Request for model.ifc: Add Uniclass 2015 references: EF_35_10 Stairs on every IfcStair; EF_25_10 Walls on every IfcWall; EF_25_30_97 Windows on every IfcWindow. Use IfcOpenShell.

First a look at what the model holds.

```python
import ifcopenshell

model = ifcopenshell.open("model.ifc")
print(model.schema)
print("classifications:", [c.Name for c in model.by_type("IfcClassification")])
for ifc_class in ("IfcDoor", "IfcRoof", "IfcStair", "IfcWall", "IfcWindow"):
    print(ifc_class, len(model.by_type(ifc_class)))
```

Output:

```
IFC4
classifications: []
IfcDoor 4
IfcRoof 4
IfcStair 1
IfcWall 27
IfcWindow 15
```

```python
import ifcopenshell
import ifcopenshell.api.classification

model = ifcopenshell.open("model.ifc")

system = ifcopenshell.api.classification.add_classification(model, classification="Uniclass 2015")

codes = {
    "IfcStair": ("EF_35_10", "Stairs"),
    "IfcWall": ("EF_25_10", "Walls"),
    "IfcWindow": ("EF_25_30_97", "Windows"),
}
for ifc_class, (code, name) in codes.items():
    products = model.by_type(ifc_class)
    ifcopenshell.api.classification.add_reference(
        model, products=products, classification=system, identification=code, name=name
    )
    print(code, len(products))

model.write("model_rev.ifc")
```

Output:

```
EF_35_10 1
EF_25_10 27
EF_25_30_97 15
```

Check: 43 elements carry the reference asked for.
